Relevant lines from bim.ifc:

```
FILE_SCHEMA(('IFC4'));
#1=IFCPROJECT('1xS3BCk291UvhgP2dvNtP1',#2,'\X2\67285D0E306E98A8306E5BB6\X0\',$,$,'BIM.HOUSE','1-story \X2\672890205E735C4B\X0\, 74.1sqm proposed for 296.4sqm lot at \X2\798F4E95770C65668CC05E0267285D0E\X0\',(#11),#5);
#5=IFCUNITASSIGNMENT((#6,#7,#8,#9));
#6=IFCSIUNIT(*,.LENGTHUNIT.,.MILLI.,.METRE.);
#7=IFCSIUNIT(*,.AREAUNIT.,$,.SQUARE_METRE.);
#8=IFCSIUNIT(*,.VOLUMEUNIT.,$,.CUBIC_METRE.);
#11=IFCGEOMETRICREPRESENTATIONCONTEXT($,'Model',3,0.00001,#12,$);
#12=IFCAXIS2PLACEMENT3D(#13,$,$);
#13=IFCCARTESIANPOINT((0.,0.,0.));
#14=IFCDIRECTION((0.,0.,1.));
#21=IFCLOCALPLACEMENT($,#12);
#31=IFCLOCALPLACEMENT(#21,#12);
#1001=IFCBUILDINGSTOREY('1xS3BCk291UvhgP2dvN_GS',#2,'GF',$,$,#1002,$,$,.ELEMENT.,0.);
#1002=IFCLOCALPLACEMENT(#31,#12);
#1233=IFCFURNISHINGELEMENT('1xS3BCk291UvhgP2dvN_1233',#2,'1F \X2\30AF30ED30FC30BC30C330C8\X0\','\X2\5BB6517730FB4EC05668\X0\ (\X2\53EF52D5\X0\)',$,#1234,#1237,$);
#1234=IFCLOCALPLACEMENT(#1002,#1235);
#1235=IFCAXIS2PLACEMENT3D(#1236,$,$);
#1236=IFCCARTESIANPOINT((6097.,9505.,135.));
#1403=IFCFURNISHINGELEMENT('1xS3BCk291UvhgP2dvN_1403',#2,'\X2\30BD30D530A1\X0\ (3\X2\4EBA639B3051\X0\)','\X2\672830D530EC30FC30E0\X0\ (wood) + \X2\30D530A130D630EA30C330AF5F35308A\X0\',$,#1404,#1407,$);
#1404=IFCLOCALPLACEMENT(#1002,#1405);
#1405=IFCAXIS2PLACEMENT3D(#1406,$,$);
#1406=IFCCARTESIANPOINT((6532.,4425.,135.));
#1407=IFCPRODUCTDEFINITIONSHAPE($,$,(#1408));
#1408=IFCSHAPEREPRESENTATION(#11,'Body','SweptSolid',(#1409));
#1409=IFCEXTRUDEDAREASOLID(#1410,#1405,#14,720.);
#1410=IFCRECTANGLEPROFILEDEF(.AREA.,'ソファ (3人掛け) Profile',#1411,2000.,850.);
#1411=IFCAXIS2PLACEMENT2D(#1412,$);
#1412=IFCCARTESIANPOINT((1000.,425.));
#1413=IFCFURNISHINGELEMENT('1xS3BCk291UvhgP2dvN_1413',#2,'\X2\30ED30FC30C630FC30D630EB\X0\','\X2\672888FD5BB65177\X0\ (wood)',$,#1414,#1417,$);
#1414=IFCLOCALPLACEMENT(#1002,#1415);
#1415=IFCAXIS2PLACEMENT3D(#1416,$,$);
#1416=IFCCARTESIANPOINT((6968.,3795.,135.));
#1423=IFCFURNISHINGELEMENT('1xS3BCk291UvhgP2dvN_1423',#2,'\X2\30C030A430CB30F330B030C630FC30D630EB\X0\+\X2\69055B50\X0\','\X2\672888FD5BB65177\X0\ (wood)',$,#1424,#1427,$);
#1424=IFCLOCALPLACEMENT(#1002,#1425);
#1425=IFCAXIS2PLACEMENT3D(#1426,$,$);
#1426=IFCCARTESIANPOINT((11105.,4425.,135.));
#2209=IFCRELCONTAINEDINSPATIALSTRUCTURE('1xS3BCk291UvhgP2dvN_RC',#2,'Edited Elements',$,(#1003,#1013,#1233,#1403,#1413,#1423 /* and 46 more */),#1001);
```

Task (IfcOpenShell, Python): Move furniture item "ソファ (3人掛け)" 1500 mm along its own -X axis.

```python
import ifcopenshell
import ifcopenshell.api.geometry
import ifcopenshell.util.placement
import ifcopenshell.util.unit

model = ifcopenshell.open("bim.ifc")
unit_scale = ifcopenshell.util.unit.calculate_unit_scale(model)

item = model.by_id(1403)
matrix = ifcopenshell.util.placement.get_local_placement(item.ObjectPlacement)
matrix[:3, 3] -= matrix[:3, 0] * 1.5 / unit_scale
ifcopenshell.api.geometry.edit_object_placement(model, product=item, matrix=matrix, is_si=False)

print(ifcopenshell.util.placement.get_local_placement(item.ObjectPlacement).round(3) + 0.0)

model.write("bim_rev.ifc")
```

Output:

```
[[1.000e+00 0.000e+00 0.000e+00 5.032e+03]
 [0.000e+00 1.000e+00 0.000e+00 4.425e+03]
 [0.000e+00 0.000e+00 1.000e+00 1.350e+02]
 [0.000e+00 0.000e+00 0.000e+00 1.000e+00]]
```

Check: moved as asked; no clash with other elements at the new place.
